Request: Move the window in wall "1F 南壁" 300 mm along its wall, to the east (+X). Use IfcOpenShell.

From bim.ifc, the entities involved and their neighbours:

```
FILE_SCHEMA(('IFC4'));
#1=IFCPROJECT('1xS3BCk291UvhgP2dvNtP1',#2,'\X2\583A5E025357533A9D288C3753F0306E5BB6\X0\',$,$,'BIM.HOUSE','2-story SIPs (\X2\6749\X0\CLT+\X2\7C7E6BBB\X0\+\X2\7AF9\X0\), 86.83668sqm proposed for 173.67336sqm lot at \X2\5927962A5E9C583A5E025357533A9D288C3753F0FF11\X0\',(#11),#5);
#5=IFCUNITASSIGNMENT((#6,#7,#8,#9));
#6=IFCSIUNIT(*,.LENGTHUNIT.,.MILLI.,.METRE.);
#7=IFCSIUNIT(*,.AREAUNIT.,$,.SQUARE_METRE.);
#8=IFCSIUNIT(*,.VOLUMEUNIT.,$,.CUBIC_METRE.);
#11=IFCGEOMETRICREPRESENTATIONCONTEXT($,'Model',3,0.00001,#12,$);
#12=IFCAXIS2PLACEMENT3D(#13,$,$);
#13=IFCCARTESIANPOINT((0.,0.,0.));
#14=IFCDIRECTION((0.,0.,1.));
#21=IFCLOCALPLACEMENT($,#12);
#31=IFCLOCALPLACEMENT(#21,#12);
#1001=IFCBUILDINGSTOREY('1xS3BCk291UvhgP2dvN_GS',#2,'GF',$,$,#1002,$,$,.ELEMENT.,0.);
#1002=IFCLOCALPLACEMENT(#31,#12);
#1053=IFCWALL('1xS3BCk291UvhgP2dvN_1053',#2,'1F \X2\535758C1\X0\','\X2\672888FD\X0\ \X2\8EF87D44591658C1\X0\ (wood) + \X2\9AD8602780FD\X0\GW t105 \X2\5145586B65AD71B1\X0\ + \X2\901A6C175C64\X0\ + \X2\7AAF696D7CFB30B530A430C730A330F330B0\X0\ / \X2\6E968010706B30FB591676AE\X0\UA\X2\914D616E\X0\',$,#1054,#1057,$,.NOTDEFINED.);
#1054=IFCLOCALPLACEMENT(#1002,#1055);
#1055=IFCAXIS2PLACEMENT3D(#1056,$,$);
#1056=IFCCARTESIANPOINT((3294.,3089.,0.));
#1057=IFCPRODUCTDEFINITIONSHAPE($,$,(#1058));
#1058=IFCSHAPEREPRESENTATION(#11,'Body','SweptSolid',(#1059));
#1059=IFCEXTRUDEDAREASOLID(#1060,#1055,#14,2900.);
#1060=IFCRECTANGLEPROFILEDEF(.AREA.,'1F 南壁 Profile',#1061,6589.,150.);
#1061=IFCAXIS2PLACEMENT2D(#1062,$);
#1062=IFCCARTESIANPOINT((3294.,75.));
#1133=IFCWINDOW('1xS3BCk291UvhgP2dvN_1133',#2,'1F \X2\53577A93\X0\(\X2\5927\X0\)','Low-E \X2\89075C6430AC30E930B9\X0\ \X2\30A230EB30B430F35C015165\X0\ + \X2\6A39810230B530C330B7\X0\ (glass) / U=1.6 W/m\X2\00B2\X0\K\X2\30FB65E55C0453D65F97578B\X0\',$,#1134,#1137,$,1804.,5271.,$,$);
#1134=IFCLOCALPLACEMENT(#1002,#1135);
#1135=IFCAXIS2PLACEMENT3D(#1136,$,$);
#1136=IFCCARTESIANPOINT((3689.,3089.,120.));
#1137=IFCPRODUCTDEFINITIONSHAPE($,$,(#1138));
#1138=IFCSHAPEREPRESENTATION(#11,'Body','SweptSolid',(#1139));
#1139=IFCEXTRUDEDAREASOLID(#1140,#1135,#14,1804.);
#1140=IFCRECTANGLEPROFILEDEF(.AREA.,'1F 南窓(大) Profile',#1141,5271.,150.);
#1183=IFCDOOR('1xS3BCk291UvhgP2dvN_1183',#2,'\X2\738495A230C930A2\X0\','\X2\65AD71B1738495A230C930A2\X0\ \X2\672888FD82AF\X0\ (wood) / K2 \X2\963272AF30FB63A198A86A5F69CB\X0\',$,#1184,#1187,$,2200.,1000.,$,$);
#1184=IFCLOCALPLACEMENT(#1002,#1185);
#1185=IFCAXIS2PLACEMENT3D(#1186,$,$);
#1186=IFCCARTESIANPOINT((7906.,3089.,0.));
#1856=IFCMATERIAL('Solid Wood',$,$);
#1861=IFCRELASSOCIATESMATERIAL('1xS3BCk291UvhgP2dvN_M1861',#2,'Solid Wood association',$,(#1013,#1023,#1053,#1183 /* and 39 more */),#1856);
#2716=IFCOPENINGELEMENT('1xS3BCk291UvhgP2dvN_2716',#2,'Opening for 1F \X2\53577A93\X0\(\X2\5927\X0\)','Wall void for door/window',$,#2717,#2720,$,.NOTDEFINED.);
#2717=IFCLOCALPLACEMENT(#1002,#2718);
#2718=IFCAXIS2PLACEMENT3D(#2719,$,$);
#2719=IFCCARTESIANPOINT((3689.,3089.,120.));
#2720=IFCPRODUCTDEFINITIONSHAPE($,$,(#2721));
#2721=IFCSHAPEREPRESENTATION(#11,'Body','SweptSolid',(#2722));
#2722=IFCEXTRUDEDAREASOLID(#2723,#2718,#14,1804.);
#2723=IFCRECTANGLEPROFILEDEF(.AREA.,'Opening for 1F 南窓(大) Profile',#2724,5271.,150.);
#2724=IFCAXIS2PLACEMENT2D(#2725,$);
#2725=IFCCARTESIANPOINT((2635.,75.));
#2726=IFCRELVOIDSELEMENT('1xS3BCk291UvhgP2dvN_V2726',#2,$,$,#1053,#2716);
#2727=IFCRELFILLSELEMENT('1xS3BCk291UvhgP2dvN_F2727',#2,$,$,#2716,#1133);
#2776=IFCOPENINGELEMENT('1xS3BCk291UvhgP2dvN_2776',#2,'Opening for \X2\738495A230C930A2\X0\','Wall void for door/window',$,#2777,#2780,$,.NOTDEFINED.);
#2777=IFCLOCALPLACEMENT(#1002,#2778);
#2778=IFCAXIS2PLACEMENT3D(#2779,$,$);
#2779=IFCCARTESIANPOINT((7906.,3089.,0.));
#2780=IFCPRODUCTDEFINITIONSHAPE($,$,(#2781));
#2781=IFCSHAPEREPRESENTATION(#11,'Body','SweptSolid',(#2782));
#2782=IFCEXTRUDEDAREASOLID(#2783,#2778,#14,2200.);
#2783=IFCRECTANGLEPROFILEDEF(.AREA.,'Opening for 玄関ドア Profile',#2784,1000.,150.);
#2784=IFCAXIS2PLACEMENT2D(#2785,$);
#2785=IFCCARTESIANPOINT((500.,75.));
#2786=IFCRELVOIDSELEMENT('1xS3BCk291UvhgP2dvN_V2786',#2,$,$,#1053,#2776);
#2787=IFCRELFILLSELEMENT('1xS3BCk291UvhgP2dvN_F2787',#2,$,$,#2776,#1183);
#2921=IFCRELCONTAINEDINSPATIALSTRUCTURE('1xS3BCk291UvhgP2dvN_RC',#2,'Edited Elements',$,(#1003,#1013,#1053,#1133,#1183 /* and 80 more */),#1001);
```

```python
import ifcopenshell
import ifcopenshell.api.geometry
import ifcopenshell.util.placement

model = ifcopenshell.open("bim.ifc")

window = model.by_guid("1xS3BCk291UvhgP2dvN_1133")
opening = window.FillsVoids[0].RelatingOpeningElement
wall = opening.VoidsElements[0].RelatingBuildingElement

wall_matrix = ifcopenshell.util.placement.get_local_placement(wall.ObjectPlacement)
shift = wall_matrix[:3, 0] * 300.0
before = ifcopenshell.util.placement.get_local_placement(window.ObjectPlacement)[:3, 3].copy()

# The window is not placed relative to its opening, so move both.
for product in (opening, window):
    matrix = ifcopenshell.util.placement.get_local_placement(product.ObjectPlacement)
    matrix[:3, 3] += shift
    ifcopenshell.api.geometry.edit_object_placement(model, product=product, matrix=matrix, is_si=False)

after = ifcopenshell.util.placement.get_local_placement(window.ObjectPlacement)[:3, 3]
print("window moved by", (after - before).round(3) + 0.0)

model.write("bim-out.ifc")
```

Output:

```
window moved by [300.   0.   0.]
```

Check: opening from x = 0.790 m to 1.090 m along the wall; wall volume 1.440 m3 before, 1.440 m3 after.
